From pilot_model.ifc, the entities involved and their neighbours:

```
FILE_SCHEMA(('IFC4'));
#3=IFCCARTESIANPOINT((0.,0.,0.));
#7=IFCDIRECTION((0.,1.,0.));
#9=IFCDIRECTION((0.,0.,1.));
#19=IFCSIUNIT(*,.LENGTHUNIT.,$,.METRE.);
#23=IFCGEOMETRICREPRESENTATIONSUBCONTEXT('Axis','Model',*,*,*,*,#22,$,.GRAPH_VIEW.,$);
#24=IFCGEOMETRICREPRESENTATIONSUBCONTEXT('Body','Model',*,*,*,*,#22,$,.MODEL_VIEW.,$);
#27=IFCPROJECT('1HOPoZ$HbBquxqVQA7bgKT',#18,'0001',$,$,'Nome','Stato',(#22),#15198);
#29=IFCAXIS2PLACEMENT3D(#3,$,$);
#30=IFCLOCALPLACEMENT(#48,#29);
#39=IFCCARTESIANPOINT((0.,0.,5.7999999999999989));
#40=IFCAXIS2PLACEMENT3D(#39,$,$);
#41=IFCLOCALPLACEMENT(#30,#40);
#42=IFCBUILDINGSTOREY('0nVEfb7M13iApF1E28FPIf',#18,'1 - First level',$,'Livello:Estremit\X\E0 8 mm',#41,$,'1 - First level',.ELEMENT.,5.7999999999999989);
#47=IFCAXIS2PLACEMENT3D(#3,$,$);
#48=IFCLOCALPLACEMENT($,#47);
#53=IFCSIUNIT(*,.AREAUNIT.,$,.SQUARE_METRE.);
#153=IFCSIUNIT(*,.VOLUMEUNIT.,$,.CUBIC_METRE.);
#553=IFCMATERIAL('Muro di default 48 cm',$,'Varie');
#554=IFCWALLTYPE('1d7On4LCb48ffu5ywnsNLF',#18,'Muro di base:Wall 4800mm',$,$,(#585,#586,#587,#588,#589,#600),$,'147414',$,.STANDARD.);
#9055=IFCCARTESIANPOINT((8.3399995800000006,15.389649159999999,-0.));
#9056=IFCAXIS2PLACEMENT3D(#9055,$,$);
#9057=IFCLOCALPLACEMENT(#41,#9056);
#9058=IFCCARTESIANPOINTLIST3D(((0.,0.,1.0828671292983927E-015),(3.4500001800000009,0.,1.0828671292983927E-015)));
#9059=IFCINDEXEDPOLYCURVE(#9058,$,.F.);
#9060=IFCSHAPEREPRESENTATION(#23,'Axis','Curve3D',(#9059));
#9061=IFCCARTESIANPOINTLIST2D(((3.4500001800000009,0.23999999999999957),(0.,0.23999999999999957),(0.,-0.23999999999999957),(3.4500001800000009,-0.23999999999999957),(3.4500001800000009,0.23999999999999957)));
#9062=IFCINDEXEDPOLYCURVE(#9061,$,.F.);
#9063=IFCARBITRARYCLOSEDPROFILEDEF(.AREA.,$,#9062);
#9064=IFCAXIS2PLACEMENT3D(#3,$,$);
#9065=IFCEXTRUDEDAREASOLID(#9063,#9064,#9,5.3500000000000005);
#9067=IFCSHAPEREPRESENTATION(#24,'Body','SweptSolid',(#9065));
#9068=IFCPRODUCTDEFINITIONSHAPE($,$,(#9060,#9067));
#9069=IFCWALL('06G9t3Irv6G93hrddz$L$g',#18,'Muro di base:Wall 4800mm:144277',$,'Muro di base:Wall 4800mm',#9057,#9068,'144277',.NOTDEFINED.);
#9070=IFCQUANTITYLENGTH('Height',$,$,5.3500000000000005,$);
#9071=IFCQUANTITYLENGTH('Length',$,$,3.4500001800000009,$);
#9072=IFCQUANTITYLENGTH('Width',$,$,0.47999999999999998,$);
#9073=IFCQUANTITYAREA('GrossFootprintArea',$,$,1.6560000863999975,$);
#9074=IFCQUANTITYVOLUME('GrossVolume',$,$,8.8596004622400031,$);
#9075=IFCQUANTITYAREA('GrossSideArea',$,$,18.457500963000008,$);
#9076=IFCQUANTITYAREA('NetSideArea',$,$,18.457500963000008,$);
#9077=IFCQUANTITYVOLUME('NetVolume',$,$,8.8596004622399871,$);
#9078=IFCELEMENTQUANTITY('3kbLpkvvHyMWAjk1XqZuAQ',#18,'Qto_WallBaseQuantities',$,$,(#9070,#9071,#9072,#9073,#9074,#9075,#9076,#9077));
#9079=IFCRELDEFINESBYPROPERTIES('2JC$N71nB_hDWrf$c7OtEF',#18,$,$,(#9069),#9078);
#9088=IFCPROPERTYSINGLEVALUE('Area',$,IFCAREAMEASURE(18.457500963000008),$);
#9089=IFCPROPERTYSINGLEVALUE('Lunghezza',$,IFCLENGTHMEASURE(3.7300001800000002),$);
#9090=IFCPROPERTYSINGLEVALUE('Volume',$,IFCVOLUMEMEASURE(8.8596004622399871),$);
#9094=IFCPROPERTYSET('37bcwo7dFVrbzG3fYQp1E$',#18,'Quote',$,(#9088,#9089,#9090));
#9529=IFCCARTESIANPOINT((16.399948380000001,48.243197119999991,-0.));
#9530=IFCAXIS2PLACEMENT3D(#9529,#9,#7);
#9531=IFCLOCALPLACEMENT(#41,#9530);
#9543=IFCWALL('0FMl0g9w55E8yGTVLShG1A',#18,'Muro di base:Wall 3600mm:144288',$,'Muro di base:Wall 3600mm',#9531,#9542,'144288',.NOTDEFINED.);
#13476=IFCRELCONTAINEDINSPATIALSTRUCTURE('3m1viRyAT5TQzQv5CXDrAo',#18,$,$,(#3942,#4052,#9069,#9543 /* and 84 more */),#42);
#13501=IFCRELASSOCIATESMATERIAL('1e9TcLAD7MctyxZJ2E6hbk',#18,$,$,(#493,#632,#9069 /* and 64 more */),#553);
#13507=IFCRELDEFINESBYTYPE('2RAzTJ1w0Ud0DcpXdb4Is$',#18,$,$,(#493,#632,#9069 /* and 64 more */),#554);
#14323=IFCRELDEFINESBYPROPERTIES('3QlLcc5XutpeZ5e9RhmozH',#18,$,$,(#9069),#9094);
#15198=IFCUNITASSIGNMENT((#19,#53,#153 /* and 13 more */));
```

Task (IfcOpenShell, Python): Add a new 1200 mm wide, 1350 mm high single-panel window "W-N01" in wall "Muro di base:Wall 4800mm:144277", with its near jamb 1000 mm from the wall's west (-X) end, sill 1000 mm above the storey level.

```python
import numpy as np
import ifcopenshell
import ifcopenshell.api.feature
import ifcopenshell.api.geometry
import ifcopenshell.api.pset
import ifcopenshell.api.root
import ifcopenshell.api.spatial
import ifcopenshell.geom
import ifcopenshell.util.element
import ifcopenshell.util.placement
import ifcopenshell.util.representation
import ifcopenshell.util.shape
import ifcopenshell.util.unit

model = ifcopenshell.open("pilot_model.ifc")
unit_scale = ifcopenshell.util.unit.calculate_unit_scale(model)
area_scale = ifcopenshell.util.unit.calculate_unit_scale(model, "AREAUNIT")
volume_scale = ifcopenshell.util.unit.calculate_unit_scale(model, "VOLUMEUNIT")
settings = ifcopenshell.geom.settings()


def volume(element):
    """Net volume in cubic metres, openings subtracted."""
    shape = ifcopenshell.geom.create_shape(settings, element)
    return ifcopenshell.util.shape.get_volume(shape.geometry)


wall = model.by_guid("06G9t3Irv6G93hrddz$L$g")
storey = ifcopenshell.util.element.get_container(wall, ifc_class="IfcBuildingStorey")
context = ifcopenshell.util.representation.get_context(model, "Model", "Body", "MODEL_VIEW")
before = volume(wall)

width, height, from_end, sill = 1.2, 1.35, 1, 1  # metres

# The wall runs along its own X axis, and the end named is its -X end.
wall_shape = ifcopenshell.geom.create_shape(settings, wall)
x, y, z = ifcopenshell.util.shape.get_vertices(wall_shape.geometry).T
start = x.min() + from_end
face, thickness = float(y.min()), float(y.max() - y.min())
wall_matrix = ifcopenshell.util.placement.get_local_placement(wall.ObjectPlacement)
level = ifcopenshell.util.placement.get_local_placement(storey.ObjectPlacement)[2, 3]


def in_wall(x, y):
    """Placement at x, y metres in the wall's axes, at sill height."""
    matrix = wall_matrix.copy()
    matrix[:, 3] = wall_matrix @ np.array([x / unit_scale, y / unit_scale, 0.0, 1.0])
    matrix[2, 3] = level + sill / unit_scale
    return matrix


# Opening: a box that overshoots both wall faces by 50 mm.
opening = ifcopenshell.api.root.create_entity(model, ifc_class="IfcOpeningElement", predefined_type="OPENING")
box = ifcopenshell.api.geometry.add_wall_representation(
    model, context=context, length=width, height=height, thickness=thickness + 0.1
)
ifcopenshell.api.geometry.assign_representation(model, product=opening, representation=box)
ifcopenshell.api.geometry.edit_object_placement(model, product=opening, matrix=in_wall(start, face - 0.05), is_si=False)
ifcopenshell.api.feature.add_feature(model, feature=opening, element=wall)

window = ifcopenshell.api.root.create_entity(model, ifc_class="IfcWindow", name="W-N01", predefined_type="WINDOW")
window.OverallWidth, window.OverallHeight = width / unit_scale, height / unit_scale
window.PartitioningType = "SINGLE_PANEL"
body = ifcopenshell.api.geometry.add_window_representation(
    model,
    context=context,
    overall_width=window.OverallWidth,
    overall_height=window.OverallHeight,
    partition_type="SINGLE_PANEL",
)
ifcopenshell.api.geometry.assign_representation(model, product=window, representation=body)
ifcopenshell.api.spatial.assign_container(model, products=[window], relating_structure=storey)
ifcopenshell.api.feature.add_filling(model, opening=opening, element=window)

# Centre the window in the wall's thickness.
ifcopenshell.api.geometry.edit_object_placement(model, product=window, matrix=in_wall(start, face), is_si=False)
window_shape = ifcopenshell.geom.create_shape(settings, window)
depth = ifcopenshell.util.shape.get_vertices(window_shape.geometry)[:, 1]
offset = face + thickness / 2 - (depth.min() + depth.max()) / 2
ifcopenshell.api.geometry.edit_object_placement(model, product=window, matrix=in_wall(start, offset), is_si=False)

after = volume(wall)

# Update the wall's stored quantities.
qto = model.by_id(ifcopenshell.util.element.get_pset(wall, "Qto_WallBaseQuantities", should_inherit=False)["id"])
ifcopenshell.api.pset.edit_qto(model, qto=qto, properties={
    "NetSideArea": after / thickness / area_scale,
    "NetVolume": after / volume_scale,
})
pset = model.by_id(ifcopenshell.util.element.get_pset(wall, "Quote", should_inherit=False)["id"])
ifcopenshell.api.pset.edit_pset(model, pset=pset, properties={
    "Area": model.create_entity("IfcAreaMeasure", after / thickness / area_scale),
    "Volume": model.create_entity("IfcVolumeMeasure", after / volume_scale),
})

print(f"wall volume {before:.3f} -> {after:.3f} m3")

model.write("pilot_model_v2.ifc")
```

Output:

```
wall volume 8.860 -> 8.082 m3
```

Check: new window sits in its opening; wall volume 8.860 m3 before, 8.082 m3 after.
